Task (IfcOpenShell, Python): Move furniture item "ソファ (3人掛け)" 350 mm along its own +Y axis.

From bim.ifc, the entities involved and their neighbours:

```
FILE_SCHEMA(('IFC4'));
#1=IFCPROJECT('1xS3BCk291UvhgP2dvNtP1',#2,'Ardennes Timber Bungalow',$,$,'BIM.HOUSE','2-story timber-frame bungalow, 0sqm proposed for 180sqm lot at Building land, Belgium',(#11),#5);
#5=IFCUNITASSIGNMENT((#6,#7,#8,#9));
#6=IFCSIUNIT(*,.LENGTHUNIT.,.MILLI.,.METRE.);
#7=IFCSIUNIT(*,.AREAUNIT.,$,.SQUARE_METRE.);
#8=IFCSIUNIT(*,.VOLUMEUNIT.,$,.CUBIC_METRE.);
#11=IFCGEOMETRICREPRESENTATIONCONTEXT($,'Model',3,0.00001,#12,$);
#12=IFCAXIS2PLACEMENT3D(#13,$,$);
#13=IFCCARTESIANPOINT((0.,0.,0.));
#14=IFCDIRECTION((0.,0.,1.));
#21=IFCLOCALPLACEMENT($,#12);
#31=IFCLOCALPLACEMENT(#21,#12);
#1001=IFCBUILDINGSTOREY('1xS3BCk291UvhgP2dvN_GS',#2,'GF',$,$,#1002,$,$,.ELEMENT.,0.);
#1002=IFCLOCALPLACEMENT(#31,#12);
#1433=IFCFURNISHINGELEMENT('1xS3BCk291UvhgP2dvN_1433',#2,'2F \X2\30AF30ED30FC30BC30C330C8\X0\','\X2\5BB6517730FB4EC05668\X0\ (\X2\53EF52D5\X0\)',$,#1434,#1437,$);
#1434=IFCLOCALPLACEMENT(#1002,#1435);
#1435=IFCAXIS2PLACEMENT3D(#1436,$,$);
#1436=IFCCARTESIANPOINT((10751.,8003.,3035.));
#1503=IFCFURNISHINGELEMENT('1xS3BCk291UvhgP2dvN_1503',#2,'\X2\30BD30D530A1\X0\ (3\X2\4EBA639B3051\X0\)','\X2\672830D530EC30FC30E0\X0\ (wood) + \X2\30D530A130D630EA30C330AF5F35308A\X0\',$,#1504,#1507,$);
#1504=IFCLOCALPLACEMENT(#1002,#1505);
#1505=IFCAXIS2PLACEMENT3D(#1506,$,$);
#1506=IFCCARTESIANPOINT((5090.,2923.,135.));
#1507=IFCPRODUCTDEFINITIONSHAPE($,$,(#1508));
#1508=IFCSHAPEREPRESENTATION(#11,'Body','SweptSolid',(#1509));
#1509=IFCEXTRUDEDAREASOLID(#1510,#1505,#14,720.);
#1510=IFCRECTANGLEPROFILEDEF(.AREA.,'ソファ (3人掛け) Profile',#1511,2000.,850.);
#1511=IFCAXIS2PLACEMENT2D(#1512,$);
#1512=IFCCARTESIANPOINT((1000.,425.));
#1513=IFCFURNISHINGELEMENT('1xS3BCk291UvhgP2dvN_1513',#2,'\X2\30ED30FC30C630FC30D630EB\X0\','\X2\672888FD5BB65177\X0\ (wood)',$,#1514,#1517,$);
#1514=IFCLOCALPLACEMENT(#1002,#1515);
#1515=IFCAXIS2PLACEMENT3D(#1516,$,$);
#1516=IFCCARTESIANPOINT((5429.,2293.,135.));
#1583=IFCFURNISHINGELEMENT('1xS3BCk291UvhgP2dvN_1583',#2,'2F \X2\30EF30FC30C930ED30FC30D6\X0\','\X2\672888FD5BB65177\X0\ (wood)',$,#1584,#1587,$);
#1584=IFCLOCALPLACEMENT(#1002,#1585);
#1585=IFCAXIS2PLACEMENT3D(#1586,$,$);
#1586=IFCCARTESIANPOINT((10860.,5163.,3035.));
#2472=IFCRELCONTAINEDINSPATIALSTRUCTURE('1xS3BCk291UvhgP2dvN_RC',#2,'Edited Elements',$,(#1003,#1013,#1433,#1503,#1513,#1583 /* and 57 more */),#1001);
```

```python
import ifcopenshell
import ifcopenshell.api.geometry
import ifcopenshell.util.placement

model = ifcopenshell.open("bim.ifc")

item = model.by_id(1503)
matrix = ifcopenshell.util.placement.get_local_placement(item.ObjectPlacement)
matrix[:3, 3] += matrix[:3, 1] * 350.0
ifcopenshell.api.geometry.edit_object_placement(model, product=item, matrix=matrix, is_si=False)

print(ifcopenshell.util.placement.get_local_placement(item.ObjectPlacement).round(3) + 0.0)

model.write("bim_v2.ifc")
```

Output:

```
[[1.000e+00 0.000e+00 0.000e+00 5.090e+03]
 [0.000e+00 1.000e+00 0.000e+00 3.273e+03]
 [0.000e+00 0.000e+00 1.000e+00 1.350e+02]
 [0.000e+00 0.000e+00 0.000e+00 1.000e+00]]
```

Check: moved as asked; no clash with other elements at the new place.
